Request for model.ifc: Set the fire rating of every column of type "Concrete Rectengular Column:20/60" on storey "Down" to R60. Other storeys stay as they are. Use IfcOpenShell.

First a look at what the model holds.

```python
import ifcopenshell
import ifcopenshell.util.element

model = ifcopenshell.open("model.ifc")
print(model.schema)
storey = next(s for s in model.by_type("IfcBuildingStorey") if s.Name == "Down")
columns = [e for e in ifcopenshell.util.element.get_decomposition(storey) if e.is_a("IfcColumn")]
seen = {}
for e in columns:
    element_type = ifcopenshell.util.element.get_type(e)
    key = (element_type.Name if element_type != e and element_type else None, ifcopenshell.util.element.get_pset(e, "Pset_ColumnCommon", "FireRating"))
    seen[key] = seen.get(key, 0) + 1
for (name, value), count in sorted(seen.items(), key=str):
    print(count, "x", name, "|", value)
```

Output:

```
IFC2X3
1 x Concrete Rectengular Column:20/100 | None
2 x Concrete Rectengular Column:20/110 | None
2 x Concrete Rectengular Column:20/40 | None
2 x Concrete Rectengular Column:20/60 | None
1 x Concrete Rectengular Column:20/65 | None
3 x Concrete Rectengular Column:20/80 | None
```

```python
import ifcopenshell
import ifcopenshell.api.pset
import ifcopenshell.util.element

model = ifcopenshell.open("model.ifc")

storey = next(s for s in model.by_type("IfcBuildingStorey") if s.Name == "Down")
columns = [e for e in ifcopenshell.util.element.get_decomposition(storey) if e.is_a("IfcColumn")]

count = 0
for e in columns:
    element_type = ifcopenshell.util.element.get_type(e)
    if element_type in (None, e) or element_type.Name != "Concrete Rectengular Column:20/60":
        continue
    # add_pset returns the element's existing set when there is one.
    pset = ifcopenshell.api.pset.add_pset(model, product=e, name="Pset_ColumnCommon")
    ifcopenshell.api.pset.edit_pset(model, pset=pset, properties={"FireRating": "R60"})
    count += 1

print(count, "columns updated")

model.write("model_edited.ifc")
```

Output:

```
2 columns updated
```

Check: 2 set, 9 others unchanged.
